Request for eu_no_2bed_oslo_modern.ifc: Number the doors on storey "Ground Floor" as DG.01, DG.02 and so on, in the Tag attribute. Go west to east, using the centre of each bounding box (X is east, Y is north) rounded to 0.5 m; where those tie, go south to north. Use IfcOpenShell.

First a look at what the model holds.

```python
import ifcopenshell
import ifcopenshell.util.element
import ifcopenshell.util.placement

model = ifcopenshell.open("eu_no_2bed_oslo_modern.ifc")
print(model.schema)
storey = next(s for s in model.by_type("IfcBuildingStorey") if s.Name == "Ground Floor")
doors = [e for e in ifcopenshell.util.element.get_decomposition(storey) if e.is_a("IfcDoor")]
for e in sorted(doors, key=lambda e: e.id()):
    origin = ifcopenshell.util.placement.get_local_placement(e.ObjectPlacement)[:3, 3]
    print(e.id(), e.Tag, e.Name, origin.round(2) + 0.0, sep=" | ")
```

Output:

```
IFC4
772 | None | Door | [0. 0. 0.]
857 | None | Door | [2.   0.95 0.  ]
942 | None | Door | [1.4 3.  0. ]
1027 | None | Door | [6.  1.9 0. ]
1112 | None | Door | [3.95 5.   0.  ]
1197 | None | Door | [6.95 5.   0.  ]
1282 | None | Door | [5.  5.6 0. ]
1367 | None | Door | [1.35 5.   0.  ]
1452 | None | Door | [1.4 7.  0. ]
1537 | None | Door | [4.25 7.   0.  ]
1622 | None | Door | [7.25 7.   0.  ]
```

```python
import ifcopenshell
import ifcopenshell.geom
import ifcopenshell.util.element
import ifcopenshell.util.shape

model = ifcopenshell.open("eu_no_2bed_oslo_modern.ifc")
settings = ifcopenshell.geom.settings()
settings.set("use-world-coords", True)


def centre(element):
    shape = ifcopenshell.geom.create_shape(settings, element)
    return ifcopenshell.util.shape.get_bbox_centroid(shape.geometry)


storey = next(s for s in model.by_type("IfcBuildingStorey") if s.Name == "Ground Floor")
doors = [e for e in ifcopenshell.util.element.get_decomposition(storey) if e.is_a("IfcDoor")]

# Insertion points can sit at a corner or the storey origin, so sort by the geometry (in metres).
centres = {e: centre(e) for e in doors}
doors.sort(key=lambda e: (round(centres[e][0] / 0.5), centres[e][1]))

for i, e in enumerate(doors, start=1):
    number = f"DG.{i:02d}"
    e.Tag = number
    print(e.id(), number)

model.write("eu_no_2bed_oslo_modern_updated.ifc")
```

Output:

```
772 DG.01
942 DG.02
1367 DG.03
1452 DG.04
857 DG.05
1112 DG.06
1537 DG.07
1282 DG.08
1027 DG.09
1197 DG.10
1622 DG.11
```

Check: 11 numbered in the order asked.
